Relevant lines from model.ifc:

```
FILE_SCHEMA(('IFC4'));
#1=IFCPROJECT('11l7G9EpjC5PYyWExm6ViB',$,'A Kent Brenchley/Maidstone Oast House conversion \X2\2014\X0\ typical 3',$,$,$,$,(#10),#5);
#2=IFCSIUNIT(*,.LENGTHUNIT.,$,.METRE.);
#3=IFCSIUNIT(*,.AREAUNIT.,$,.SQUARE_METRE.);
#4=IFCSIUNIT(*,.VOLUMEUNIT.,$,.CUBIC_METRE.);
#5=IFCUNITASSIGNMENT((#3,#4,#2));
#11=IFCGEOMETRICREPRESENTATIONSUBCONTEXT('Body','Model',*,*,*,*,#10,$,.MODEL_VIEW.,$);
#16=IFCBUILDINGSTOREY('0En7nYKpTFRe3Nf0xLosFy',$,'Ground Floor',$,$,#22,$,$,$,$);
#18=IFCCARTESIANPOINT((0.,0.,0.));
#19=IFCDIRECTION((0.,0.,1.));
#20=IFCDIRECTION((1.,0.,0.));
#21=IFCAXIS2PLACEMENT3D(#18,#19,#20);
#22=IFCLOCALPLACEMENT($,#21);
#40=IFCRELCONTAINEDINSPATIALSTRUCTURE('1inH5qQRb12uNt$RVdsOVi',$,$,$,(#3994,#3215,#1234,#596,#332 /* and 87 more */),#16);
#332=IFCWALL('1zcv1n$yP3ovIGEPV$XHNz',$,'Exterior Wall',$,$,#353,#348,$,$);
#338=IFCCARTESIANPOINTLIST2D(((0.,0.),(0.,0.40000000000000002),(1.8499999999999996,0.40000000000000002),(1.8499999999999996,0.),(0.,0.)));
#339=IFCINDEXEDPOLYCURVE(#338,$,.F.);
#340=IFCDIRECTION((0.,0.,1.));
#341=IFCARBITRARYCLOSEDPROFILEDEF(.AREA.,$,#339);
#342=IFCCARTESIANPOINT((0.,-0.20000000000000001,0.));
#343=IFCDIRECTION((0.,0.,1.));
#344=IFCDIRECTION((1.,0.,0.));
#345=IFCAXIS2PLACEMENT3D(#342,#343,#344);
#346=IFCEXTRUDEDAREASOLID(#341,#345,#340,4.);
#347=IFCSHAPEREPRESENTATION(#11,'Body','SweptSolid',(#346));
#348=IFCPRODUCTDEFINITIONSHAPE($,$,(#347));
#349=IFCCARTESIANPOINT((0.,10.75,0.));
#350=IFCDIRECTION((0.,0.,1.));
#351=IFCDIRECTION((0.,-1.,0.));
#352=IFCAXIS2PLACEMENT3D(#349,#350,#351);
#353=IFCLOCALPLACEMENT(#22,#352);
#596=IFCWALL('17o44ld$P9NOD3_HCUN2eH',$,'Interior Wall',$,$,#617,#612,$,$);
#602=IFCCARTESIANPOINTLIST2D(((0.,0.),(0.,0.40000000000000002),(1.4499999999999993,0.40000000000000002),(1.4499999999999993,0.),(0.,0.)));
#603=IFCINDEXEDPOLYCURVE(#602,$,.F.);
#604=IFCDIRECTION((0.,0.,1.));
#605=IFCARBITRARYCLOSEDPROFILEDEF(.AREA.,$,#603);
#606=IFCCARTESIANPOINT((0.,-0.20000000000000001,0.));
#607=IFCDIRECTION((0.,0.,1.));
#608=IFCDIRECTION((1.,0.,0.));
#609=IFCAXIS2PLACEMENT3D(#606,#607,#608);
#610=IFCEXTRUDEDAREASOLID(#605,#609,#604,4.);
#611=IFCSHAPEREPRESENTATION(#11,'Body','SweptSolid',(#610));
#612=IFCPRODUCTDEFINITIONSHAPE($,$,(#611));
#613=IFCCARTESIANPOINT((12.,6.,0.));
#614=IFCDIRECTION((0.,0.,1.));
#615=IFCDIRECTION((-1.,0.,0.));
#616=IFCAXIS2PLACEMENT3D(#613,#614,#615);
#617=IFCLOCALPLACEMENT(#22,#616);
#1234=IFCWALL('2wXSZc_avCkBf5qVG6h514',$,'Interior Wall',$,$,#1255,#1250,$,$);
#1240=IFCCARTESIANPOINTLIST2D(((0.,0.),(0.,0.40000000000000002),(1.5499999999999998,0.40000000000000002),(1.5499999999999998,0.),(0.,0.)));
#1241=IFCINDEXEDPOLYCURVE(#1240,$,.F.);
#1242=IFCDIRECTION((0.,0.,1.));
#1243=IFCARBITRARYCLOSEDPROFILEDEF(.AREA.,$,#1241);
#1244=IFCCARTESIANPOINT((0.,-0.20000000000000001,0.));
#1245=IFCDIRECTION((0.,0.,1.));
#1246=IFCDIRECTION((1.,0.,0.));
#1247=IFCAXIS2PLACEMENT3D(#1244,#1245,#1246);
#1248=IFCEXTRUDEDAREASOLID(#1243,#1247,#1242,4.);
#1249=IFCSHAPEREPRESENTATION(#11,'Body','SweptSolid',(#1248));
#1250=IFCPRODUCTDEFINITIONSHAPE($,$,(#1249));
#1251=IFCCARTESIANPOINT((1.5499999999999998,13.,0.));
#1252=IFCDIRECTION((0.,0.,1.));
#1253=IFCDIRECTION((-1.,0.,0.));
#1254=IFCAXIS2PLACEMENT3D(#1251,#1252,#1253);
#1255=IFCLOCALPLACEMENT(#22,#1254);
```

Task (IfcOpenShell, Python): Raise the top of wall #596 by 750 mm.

```python
import ifcopenshell
import ifcopenshell.geom
import ifcopenshell.util.representation
import ifcopenshell.util.shape

model = ifcopenshell.open("model.ifc")
settings = ifcopenshell.geom.settings()


def volume(element):
    """Net volume in cubic metres, openings subtracted."""
    shape = ifcopenshell.geom.create_shape(settings, element)
    return ifcopenshell.util.shape.get_volume(shape.geometry)


wall = model.by_guid("17o44ld$P9NOD3_HCUN2eH")
before = volume(wall)

body = ifcopenshell.util.representation.get_representation(wall, "Model", "Body")
solid = body.Items[0]
old_height = solid.Depth
solid.Depth += 0.75
after = volume(wall)

print(f"height {old_height:g} -> {solid.Depth:g}, volume {before:.3f} -> {after:.3f} m3")

model.write("model_rev.ifc")
```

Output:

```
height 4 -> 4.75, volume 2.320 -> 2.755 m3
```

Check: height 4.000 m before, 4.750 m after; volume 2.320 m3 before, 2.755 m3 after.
